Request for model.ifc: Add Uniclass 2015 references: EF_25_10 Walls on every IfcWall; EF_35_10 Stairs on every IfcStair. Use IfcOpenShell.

First a look at what the model holds.

```python
import ifcopenshell

model = ifcopenshell.open("model.ifc")
print(model.schema)
print("classifications:", [c.Name for c in model.by_type("IfcClassification")])
for ifc_class in ("IfcDoor", "IfcRoof", "IfcStair", "IfcWall", "IfcWindow"):
    print(ifc_class, len(model.by_type(ifc_class)))
```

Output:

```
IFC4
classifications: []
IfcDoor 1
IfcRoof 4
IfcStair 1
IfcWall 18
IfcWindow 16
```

```python
import ifcopenshell
import ifcopenshell.api.classification

model = ifcopenshell.open("model.ifc")

system = ifcopenshell.api.classification.add_classification(model, classification="Uniclass 2015")

codes = {
    "IfcWall": ("EF_25_10", "Walls"),
    "IfcStair": ("EF_35_10", "Stairs"),
}
for ifc_class, (code, name) in codes.items():
    products = model.by_type(ifc_class)
    ifcopenshell.api.classification.add_reference(
        model, products=products, classification=system, identification=code, name=name
    )
    print(code, len(products))

model.write("model-out.ifc")
```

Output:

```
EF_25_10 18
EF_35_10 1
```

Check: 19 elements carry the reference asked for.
